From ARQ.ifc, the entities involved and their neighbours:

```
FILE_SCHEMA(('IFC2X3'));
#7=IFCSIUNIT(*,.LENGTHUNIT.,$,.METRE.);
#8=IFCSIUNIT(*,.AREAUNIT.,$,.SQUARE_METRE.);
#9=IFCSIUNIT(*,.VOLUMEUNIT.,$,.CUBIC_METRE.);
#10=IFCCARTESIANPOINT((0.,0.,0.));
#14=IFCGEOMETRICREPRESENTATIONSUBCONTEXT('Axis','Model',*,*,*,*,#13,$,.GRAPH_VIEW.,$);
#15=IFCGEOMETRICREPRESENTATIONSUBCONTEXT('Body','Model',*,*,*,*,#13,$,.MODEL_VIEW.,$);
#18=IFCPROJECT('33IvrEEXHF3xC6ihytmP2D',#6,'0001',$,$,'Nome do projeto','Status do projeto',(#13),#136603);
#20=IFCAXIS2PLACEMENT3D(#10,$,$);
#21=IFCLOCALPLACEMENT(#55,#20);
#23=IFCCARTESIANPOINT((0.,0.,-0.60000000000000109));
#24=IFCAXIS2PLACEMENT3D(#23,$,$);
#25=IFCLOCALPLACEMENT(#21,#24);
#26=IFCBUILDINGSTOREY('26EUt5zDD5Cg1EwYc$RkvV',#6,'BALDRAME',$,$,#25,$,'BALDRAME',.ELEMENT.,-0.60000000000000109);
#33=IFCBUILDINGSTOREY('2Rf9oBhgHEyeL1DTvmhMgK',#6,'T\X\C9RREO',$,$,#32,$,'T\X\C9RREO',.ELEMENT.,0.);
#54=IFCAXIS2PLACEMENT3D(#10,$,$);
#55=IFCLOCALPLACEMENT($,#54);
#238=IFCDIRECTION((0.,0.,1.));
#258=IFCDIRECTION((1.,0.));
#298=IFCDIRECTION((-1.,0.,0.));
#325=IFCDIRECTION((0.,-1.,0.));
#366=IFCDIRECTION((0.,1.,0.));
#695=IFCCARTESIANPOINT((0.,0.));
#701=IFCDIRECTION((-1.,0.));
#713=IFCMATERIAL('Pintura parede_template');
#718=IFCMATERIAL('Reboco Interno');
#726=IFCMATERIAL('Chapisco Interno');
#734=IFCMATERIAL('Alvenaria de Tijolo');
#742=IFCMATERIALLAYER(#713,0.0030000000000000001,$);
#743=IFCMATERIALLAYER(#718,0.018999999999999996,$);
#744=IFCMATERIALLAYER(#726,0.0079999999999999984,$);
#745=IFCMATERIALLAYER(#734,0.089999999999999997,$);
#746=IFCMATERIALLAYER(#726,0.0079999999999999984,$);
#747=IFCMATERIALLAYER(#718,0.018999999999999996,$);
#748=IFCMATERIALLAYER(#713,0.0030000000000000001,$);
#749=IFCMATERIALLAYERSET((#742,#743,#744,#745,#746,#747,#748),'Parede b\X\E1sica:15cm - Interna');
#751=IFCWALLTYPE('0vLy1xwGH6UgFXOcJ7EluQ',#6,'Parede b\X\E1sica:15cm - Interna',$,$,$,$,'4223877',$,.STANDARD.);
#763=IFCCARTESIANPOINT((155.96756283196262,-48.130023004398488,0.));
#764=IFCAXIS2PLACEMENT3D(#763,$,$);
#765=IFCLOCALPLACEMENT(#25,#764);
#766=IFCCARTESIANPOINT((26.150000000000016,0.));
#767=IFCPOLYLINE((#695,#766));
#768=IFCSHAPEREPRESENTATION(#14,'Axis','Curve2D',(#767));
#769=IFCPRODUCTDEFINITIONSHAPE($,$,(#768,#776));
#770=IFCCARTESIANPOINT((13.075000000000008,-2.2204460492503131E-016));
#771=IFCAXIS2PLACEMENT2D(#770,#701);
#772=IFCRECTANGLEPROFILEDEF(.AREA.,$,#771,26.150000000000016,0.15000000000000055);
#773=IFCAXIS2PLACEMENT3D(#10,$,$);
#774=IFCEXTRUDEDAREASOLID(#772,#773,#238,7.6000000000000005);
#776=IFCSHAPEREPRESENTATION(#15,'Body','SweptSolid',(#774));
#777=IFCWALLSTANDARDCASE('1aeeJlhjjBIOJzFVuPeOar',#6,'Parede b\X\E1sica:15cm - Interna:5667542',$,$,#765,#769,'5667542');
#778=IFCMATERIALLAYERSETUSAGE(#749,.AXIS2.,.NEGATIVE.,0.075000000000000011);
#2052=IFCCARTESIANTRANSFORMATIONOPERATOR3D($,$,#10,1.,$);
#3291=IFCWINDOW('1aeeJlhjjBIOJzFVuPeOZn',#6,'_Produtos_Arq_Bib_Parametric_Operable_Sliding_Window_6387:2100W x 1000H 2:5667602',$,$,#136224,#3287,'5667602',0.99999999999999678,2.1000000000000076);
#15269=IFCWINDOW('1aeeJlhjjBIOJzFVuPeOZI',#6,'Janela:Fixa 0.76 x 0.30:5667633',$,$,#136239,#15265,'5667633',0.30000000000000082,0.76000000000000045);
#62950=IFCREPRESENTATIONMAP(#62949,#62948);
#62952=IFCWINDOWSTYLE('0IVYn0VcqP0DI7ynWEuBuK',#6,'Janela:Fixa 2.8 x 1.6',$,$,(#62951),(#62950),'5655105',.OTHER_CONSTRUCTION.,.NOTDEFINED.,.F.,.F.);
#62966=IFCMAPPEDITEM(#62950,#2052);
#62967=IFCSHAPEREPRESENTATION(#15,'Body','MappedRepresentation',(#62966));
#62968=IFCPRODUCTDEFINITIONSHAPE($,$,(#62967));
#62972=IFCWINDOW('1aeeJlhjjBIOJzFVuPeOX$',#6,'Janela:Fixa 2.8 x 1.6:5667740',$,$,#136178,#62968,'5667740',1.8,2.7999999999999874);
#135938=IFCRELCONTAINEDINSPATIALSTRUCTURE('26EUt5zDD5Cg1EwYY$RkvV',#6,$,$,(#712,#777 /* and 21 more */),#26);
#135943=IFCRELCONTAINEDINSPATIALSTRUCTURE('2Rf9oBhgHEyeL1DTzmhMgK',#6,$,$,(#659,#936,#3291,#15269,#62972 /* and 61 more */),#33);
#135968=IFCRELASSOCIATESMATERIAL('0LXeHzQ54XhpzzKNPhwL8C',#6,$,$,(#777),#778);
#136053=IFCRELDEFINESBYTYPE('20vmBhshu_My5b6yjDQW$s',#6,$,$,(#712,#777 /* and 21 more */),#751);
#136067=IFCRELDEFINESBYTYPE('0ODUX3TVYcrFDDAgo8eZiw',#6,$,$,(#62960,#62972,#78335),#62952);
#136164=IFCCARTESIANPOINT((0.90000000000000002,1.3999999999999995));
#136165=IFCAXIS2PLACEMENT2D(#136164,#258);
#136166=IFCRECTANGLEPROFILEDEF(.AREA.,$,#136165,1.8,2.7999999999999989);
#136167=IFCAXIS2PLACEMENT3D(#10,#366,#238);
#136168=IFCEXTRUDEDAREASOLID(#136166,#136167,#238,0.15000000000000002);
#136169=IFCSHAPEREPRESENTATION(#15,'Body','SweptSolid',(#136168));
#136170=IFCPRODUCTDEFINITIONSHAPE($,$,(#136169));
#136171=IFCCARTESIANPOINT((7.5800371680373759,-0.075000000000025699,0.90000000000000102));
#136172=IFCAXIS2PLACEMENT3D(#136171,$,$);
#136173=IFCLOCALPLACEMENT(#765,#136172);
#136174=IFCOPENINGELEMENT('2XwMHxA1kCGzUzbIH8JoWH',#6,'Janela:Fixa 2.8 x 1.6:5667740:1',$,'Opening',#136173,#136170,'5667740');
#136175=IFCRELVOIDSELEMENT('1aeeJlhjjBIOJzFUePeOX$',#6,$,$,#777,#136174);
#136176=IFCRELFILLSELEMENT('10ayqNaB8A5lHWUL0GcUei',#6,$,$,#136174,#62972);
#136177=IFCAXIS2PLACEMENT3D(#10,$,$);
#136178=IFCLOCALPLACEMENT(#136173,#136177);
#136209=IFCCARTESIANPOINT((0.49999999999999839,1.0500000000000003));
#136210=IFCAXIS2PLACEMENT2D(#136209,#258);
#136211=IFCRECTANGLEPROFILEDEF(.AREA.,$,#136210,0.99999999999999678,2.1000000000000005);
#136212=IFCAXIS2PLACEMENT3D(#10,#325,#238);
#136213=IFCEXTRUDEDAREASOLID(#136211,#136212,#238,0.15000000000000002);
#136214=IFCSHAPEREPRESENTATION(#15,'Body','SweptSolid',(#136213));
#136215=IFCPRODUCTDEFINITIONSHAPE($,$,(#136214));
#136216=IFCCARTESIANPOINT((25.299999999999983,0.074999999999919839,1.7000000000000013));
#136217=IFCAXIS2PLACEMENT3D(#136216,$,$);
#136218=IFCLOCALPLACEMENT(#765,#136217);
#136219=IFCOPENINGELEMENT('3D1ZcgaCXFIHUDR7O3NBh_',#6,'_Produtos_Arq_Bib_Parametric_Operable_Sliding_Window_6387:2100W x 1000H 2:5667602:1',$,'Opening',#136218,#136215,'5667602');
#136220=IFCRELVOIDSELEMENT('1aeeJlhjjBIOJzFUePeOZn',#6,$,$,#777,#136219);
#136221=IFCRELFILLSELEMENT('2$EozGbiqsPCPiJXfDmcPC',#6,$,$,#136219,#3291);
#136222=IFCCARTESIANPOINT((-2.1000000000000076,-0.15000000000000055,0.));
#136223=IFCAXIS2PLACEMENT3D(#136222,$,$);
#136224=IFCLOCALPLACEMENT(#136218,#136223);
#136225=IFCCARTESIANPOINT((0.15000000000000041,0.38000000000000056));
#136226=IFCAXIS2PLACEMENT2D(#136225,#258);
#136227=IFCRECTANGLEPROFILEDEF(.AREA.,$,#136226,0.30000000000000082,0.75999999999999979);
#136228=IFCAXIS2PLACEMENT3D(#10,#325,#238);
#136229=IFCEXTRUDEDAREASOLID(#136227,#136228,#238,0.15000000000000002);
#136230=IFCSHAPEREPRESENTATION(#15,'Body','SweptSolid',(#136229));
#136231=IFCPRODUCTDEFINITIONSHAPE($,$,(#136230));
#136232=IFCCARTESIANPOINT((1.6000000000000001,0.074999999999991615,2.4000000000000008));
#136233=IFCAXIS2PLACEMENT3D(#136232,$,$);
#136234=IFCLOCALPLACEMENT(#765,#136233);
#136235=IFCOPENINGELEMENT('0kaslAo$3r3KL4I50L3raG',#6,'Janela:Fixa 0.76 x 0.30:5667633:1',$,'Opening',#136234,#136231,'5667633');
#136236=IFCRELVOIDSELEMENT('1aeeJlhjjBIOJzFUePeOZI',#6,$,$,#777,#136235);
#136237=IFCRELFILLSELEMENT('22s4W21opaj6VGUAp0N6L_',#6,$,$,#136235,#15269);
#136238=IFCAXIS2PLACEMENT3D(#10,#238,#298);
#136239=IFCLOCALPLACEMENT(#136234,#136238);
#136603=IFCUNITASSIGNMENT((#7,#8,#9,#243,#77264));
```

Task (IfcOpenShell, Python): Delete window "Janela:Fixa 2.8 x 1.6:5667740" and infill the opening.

```python
import ifcopenshell
import ifcopenshell.api.feature
import ifcopenshell.api.root
import ifcopenshell.geom
import ifcopenshell.util.shape

model = ifcopenshell.open("ARQ.ifc")
settings = ifcopenshell.geom.settings()


def volume(element):
    """Net volume in cubic metres, openings subtracted."""
    shape = ifcopenshell.geom.create_shape(settings, element)
    return ifcopenshell.util.shape.get_volume(shape.geometry)


window = model.by_guid("1aeeJlhjjBIOJzFVuPeOX$")
opening = window.FillsVoids[0].RelatingOpeningElement
wall = opening.VoidsElements[0].RelatingBuildingElement
before = volume(wall)

ifcopenshell.api.root.remove_product(model, product=window)
ifcopenshell.api.feature.remove_feature(model, feature=opening)

after = volume(wall)

print(f"wall volume {before:.3f} -> {after:.3f} m3")

model.write("ARQ-out.ifc")
```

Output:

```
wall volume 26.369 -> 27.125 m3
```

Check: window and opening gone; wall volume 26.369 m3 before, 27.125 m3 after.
